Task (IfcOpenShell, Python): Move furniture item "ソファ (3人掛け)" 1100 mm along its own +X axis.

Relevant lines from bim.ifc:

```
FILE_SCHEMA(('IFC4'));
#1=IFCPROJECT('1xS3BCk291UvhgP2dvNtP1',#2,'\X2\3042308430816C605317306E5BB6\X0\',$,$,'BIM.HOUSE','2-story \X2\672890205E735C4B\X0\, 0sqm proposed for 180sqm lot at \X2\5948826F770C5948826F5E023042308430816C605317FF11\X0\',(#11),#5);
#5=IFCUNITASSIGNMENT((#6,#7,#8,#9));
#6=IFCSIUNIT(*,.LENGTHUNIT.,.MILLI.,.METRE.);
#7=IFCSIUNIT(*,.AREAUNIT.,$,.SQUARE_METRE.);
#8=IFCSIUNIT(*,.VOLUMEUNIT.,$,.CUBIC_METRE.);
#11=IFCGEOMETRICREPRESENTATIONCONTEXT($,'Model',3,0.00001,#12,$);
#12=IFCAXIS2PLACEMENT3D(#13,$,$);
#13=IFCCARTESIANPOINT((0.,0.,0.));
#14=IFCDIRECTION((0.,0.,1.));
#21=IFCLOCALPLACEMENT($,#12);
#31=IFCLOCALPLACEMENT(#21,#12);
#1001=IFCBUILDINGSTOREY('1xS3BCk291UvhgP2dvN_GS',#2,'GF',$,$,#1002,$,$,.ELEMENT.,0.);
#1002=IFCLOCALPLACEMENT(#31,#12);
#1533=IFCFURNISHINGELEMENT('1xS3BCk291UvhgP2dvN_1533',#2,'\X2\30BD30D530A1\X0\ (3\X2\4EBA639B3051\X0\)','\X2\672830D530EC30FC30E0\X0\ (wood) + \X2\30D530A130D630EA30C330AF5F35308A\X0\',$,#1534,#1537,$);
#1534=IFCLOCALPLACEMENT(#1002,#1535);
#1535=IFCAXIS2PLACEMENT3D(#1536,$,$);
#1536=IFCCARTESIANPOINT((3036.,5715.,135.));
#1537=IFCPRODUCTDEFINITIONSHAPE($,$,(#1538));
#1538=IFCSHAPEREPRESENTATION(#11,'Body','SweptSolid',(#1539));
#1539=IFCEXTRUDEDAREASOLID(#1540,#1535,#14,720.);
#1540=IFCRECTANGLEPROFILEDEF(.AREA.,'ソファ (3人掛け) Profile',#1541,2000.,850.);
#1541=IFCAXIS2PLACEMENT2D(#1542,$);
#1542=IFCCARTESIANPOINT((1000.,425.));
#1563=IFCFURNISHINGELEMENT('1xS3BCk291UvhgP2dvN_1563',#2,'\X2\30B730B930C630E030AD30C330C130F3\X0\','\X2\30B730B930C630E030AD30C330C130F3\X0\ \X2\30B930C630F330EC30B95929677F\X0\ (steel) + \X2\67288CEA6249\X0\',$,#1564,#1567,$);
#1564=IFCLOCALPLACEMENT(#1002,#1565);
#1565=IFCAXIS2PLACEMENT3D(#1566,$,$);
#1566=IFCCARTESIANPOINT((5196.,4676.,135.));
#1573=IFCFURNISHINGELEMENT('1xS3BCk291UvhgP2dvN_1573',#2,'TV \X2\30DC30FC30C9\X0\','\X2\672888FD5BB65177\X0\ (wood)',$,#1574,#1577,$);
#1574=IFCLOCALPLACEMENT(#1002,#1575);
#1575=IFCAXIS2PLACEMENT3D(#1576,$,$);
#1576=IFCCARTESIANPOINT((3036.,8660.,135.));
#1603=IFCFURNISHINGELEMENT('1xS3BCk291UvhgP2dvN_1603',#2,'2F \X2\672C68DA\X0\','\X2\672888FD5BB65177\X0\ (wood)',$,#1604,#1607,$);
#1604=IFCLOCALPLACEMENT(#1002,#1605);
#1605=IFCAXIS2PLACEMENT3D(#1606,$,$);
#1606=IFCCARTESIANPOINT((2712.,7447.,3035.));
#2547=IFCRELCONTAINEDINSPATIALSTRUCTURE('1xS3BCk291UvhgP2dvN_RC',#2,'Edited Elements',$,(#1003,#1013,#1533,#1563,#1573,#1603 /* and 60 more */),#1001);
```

```python
import ifcopenshell
import ifcopenshell.api.geometry
import ifcopenshell.util.placement
import ifcopenshell.util.unit

model = ifcopenshell.open("bim.ifc")
unit_scale = ifcopenshell.util.unit.calculate_unit_scale(model)

item = model.by_guid("1xS3BCk291UvhgP2dvN_1533")
matrix = ifcopenshell.util.placement.get_local_placement(item.ObjectPlacement)
matrix[:3, 3] += matrix[:3, 0] * 1.1 / unit_scale
ifcopenshell.api.geometry.edit_object_placement(model, product=item, matrix=matrix, is_si=False)

print(ifcopenshell.util.placement.get_local_placement(item.ObjectPlacement).round(3) + 0.0)

model.write("bim_updated.ifc")
```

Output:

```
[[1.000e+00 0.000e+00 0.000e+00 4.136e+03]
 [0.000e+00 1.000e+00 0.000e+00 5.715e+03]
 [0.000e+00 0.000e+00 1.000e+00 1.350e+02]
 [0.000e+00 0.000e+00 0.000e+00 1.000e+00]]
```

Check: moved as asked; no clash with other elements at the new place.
